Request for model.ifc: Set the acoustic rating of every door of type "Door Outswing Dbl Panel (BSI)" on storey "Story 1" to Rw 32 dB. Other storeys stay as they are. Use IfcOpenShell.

First a look at what the model holds.

```python
import ifcopenshell
import ifcopenshell.util.element

model = ifcopenshell.open("model.ifc")
print(model.schema)
storey = next(s for s in model.by_type("IfcBuildingStorey") if s.Name == "Story 1")
doors = [e for e in ifcopenshell.util.element.get_decomposition(storey) if e.is_a("IfcDoor")]
seen = {}
for e in doors:
    element_type = ifcopenshell.util.element.get_type(e)
    key = (element_type.Name if element_type != e and element_type else None, ifcopenshell.util.element.get_pset(e, "Pset_DoorCommon", "AcousticRating"))
    seen[key] = seen.get(key, 0) + 1
for (name, value), count in sorted(seen.items(), key=str):
    print(count, "x", name, "|", value)
```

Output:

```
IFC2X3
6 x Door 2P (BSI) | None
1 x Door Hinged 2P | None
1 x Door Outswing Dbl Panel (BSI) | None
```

```python
import ifcopenshell
import ifcopenshell.api.pset
import ifcopenshell.util.element

model = ifcopenshell.open("model.ifc")

storey = next(s for s in model.by_type("IfcBuildingStorey") if s.Name == "Story 1")
doors = [e for e in ifcopenshell.util.element.get_decomposition(storey) if e.is_a("IfcDoor")]

count = 0
for e in doors:
    element_type = ifcopenshell.util.element.get_type(e)
    if element_type in (None, e) or element_type.Name != "Door Outswing Dbl Panel (BSI)":
        continue
    # add_pset returns the element's existing set when there is one.
    pset = ifcopenshell.api.pset.add_pset(model, product=e, name="Pset_DoorCommon")
    ifcopenshell.api.pset.edit_pset(model, pset=pset, properties={"AcousticRating": "Rw 32 dB"})
    count += 1

print(count, "doors updated")

model.write("model_v2.ifc")
```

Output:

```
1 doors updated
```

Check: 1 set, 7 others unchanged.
